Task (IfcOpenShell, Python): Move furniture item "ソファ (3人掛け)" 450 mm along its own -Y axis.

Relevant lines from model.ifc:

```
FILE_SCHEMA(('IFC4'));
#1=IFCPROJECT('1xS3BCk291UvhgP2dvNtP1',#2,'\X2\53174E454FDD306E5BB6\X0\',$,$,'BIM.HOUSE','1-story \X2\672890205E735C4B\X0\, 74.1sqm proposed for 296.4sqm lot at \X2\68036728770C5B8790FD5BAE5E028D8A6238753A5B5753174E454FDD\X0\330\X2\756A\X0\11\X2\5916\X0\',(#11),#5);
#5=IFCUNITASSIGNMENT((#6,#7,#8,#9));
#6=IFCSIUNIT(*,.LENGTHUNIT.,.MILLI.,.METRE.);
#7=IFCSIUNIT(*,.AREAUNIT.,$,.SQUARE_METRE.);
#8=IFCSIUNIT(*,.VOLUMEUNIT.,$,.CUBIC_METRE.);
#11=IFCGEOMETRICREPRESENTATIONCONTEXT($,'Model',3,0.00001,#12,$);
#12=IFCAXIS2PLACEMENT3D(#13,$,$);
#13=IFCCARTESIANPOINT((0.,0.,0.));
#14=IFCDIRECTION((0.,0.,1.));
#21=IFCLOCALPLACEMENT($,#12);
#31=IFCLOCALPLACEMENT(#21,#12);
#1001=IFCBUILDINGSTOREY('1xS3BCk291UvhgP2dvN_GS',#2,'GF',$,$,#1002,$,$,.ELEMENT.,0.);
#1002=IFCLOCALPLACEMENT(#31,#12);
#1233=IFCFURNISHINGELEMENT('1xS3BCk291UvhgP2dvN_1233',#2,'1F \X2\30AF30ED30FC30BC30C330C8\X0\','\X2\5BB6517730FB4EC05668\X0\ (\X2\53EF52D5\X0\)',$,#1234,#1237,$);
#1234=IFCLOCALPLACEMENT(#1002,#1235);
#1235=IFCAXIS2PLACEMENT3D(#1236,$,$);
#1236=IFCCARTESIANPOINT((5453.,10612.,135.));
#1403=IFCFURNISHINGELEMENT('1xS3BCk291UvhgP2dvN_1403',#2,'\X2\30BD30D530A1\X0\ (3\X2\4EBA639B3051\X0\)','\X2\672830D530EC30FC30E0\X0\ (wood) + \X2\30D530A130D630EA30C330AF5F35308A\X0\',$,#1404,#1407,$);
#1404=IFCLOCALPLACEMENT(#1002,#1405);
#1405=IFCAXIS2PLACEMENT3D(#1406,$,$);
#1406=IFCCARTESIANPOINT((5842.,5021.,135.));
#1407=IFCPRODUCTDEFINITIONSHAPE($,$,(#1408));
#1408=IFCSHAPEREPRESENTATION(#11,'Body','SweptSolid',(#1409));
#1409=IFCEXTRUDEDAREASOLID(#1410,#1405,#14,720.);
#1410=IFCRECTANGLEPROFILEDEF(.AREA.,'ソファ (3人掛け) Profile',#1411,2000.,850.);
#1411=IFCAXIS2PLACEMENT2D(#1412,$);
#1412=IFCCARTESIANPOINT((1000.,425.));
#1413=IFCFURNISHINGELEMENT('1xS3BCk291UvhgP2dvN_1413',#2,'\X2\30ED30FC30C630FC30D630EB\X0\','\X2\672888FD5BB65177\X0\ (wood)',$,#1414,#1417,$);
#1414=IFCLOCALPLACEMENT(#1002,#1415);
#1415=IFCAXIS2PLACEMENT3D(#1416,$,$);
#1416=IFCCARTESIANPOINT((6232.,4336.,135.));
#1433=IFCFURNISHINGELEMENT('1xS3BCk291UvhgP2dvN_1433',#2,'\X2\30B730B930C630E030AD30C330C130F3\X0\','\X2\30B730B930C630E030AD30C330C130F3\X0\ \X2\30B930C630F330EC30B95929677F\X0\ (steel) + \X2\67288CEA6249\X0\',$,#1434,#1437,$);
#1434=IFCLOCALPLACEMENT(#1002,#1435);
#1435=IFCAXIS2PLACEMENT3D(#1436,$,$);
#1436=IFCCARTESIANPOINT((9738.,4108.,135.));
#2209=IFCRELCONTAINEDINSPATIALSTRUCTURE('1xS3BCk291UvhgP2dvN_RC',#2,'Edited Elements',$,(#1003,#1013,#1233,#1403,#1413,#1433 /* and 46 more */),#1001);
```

```python
import ifcopenshell
import ifcopenshell.api.geometry
import ifcopenshell.util.placement

model = ifcopenshell.open("model.ifc")

item = model.by_id(1403)
matrix = ifcopenshell.util.placement.get_local_placement(item.ObjectPlacement)
matrix[:3, 3] -= matrix[:3, 1] * 450.0
ifcopenshell.api.geometry.edit_object_placement(model, product=item, matrix=matrix, is_si=False)

print(ifcopenshell.util.placement.get_local_placement(item.ObjectPlacement).round(3) + 0.0)

model.write("model_edited.ifc")
```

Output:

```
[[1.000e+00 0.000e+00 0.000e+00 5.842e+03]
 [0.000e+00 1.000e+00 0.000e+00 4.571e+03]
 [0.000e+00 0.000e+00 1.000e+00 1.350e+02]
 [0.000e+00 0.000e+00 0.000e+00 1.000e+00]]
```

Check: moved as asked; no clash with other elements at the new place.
